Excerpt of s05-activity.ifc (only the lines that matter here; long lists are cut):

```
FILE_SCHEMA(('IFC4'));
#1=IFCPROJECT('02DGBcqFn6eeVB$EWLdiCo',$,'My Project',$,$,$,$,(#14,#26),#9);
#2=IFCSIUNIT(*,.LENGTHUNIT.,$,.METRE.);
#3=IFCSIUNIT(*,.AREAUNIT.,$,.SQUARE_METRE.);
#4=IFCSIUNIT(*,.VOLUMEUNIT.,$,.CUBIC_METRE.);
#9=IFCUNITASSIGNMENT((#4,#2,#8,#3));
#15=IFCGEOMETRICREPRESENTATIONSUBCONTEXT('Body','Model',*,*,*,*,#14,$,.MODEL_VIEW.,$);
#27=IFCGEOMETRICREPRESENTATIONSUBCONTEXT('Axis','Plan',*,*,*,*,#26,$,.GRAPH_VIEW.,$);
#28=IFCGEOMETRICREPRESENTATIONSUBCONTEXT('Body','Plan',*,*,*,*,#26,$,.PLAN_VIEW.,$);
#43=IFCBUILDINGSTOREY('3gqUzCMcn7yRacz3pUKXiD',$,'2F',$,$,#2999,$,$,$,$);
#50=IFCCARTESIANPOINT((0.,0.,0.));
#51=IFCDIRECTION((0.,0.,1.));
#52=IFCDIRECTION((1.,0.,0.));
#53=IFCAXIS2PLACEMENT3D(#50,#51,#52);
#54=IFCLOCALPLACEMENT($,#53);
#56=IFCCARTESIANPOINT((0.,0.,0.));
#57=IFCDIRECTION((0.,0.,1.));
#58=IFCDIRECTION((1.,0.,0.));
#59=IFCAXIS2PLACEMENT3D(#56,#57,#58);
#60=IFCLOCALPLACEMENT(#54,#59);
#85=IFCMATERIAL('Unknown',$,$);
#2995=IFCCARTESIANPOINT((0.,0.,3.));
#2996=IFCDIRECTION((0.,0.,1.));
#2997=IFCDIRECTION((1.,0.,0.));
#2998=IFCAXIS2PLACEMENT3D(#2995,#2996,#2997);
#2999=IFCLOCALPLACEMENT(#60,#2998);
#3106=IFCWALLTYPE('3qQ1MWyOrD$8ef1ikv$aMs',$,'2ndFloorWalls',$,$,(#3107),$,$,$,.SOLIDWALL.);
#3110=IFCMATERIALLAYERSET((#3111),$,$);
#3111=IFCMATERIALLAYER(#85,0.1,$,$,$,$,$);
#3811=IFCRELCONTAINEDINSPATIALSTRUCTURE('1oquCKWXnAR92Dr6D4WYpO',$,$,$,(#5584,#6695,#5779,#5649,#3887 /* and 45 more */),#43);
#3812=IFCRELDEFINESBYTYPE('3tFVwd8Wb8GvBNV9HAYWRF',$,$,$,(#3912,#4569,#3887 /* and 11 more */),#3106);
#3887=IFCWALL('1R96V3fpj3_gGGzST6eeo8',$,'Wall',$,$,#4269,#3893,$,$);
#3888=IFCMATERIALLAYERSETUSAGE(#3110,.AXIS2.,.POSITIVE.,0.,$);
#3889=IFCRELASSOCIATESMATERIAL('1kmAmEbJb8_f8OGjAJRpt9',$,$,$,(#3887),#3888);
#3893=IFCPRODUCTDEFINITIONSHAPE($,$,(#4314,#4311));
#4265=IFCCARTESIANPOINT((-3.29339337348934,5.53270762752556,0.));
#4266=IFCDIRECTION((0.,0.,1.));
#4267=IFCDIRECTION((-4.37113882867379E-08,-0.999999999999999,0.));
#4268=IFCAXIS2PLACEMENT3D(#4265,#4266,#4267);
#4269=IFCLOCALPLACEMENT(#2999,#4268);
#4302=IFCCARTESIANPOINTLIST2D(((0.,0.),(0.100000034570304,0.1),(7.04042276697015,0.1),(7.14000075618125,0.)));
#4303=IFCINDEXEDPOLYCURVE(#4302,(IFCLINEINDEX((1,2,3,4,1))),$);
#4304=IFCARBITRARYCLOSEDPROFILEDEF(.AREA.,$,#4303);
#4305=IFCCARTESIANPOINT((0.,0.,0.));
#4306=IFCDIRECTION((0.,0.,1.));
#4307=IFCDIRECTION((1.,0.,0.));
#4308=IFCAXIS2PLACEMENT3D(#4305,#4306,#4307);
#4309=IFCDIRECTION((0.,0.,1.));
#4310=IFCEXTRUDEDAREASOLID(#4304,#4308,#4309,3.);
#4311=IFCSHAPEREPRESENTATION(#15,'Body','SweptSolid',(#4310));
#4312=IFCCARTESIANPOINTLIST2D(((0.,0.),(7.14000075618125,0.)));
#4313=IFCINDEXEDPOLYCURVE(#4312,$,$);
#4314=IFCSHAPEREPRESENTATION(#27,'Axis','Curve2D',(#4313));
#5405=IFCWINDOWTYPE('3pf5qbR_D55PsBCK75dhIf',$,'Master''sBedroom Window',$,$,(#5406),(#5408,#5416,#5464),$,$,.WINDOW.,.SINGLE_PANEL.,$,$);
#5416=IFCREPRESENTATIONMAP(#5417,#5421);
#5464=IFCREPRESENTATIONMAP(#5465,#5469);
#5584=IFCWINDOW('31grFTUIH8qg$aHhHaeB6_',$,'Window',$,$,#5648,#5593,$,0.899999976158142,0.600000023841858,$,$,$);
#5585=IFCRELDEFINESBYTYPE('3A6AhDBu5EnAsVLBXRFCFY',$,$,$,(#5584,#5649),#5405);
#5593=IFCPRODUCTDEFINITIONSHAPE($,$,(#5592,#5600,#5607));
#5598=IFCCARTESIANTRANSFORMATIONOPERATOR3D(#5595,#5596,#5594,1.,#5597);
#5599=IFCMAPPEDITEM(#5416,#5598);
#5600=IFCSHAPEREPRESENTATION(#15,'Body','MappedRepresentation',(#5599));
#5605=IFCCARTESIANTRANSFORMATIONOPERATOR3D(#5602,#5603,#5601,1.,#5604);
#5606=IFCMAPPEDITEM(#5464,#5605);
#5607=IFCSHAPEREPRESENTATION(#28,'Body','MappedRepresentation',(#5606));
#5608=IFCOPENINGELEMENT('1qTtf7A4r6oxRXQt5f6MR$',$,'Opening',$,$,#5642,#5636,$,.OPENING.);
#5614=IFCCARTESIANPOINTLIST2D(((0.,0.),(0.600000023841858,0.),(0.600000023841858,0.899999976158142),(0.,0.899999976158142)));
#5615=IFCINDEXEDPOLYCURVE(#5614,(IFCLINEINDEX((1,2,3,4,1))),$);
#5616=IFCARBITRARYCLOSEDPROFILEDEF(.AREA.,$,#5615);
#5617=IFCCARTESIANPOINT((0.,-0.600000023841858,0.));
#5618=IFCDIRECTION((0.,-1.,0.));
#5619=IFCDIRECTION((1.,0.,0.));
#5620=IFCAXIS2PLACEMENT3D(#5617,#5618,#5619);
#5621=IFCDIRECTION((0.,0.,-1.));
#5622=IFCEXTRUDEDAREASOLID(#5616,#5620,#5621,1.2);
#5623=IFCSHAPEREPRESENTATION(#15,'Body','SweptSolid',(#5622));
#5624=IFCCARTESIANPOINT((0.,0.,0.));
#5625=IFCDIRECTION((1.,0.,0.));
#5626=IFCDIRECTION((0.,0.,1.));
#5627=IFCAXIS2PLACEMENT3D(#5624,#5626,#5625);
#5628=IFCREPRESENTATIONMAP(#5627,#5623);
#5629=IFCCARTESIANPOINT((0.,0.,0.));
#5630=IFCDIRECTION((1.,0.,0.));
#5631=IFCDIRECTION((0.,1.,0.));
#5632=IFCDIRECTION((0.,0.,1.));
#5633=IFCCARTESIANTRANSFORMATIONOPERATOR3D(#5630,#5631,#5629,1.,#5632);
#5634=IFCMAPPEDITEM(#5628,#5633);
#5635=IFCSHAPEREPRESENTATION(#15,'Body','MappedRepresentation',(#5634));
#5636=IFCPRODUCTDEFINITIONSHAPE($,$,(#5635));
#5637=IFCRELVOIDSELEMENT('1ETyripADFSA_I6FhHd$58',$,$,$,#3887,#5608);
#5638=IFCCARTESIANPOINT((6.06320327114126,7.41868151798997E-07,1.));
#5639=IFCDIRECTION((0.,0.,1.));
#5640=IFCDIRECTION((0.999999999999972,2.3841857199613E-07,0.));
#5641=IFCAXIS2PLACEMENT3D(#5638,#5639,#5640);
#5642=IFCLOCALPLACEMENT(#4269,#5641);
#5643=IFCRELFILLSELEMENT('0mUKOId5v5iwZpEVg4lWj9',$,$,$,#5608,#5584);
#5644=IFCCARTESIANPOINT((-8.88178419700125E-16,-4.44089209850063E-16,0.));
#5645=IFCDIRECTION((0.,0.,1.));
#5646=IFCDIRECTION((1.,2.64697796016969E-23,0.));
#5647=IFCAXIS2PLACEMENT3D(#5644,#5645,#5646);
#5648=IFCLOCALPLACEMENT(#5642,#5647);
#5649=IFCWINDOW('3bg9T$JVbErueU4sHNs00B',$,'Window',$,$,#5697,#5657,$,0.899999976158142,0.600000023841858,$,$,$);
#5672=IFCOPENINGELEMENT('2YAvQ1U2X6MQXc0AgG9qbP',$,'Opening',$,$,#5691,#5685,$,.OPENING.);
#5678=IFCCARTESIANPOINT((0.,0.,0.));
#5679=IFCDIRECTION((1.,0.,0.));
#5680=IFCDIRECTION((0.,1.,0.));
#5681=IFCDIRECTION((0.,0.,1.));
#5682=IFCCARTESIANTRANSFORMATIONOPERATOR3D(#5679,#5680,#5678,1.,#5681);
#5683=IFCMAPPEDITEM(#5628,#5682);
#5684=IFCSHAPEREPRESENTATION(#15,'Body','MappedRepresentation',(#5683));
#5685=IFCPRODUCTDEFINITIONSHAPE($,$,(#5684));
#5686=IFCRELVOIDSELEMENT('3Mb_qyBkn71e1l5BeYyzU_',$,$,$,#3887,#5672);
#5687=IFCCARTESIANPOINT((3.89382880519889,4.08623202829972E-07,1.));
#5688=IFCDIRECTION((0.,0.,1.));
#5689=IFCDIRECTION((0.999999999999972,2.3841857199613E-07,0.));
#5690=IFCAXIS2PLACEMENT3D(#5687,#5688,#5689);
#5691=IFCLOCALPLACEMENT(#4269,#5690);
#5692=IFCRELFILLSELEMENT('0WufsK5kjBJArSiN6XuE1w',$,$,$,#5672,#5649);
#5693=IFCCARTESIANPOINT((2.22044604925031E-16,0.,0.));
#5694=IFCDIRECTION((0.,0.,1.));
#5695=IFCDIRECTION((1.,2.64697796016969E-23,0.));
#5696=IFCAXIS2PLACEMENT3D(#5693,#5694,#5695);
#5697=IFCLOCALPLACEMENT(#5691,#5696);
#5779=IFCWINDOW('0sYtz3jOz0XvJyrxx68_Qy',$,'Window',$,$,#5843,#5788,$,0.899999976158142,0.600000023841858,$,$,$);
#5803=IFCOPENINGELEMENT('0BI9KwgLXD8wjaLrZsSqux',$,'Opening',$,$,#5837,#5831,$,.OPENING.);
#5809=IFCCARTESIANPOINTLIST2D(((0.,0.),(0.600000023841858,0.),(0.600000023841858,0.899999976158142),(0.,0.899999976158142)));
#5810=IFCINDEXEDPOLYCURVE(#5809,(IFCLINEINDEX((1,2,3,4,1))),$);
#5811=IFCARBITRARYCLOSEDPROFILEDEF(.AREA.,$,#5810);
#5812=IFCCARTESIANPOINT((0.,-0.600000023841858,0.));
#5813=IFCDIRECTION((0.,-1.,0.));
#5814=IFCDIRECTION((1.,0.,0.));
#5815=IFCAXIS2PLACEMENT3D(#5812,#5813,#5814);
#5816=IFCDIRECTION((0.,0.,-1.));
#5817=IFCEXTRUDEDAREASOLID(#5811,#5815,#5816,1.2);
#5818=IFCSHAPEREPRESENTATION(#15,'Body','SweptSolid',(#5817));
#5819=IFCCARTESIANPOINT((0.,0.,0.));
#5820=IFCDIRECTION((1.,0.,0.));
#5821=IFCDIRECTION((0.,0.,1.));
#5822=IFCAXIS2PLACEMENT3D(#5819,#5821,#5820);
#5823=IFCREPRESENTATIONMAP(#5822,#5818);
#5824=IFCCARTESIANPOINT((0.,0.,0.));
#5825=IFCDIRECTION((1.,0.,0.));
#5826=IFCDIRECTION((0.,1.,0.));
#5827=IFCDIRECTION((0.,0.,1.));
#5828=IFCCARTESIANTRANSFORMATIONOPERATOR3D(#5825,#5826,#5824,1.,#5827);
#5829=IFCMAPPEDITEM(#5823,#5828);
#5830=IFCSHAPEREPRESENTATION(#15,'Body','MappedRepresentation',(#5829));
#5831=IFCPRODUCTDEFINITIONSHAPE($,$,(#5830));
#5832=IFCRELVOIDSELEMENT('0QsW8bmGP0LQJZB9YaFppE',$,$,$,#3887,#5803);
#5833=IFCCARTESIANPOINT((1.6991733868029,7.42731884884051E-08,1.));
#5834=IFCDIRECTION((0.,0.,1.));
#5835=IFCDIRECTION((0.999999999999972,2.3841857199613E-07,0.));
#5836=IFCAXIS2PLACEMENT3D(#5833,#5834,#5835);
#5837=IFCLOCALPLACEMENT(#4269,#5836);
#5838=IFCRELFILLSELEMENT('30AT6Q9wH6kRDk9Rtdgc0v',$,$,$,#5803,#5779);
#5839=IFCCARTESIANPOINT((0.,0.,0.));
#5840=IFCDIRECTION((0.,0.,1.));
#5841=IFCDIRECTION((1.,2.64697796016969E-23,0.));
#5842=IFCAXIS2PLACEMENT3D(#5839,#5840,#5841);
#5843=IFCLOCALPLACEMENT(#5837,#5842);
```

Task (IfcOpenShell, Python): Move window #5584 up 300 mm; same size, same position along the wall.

```python
import numpy as np
import ifcopenshell
import ifcopenshell.api.geometry
import ifcopenshell.util.placement
import ifcopenshell.util.unit

model = ifcopenshell.open("s05-activity.ifc")
unit_scale = ifcopenshell.util.unit.calculate_unit_scale(model)

window = model.by_guid("31grFTUIH8qg$aHhHaeB6_")
opening = window.FillsVoids[0].RelatingOpeningElement
dz = 0.3

shift = np.array([0.0, 0.0, dz])
# The window is placed relative to its opening, so it follows when the opening moves.
matrix = ifcopenshell.util.placement.get_local_placement(opening.ObjectPlacement)
matrix[:3, 3] += shift
ifcopenshell.api.geometry.edit_object_placement(
    model, product=opening, matrix=matrix, is_si=False, should_transform_children=True
)

print(f"moved by {dz * unit_scale:+.3f} m")

model.write("s05-activity_edited.ifc")
```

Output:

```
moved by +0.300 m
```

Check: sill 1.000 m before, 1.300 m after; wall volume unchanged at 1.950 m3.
